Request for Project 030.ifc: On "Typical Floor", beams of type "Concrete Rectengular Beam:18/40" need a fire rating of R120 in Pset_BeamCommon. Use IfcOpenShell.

First a look at what the model holds.

```python
import ifcopenshell
import ifcopenshell.util.element

model = ifcopenshell.open("Project 030.ifc")
print(model.schema)
storey = next(s for s in model.by_type("IfcBuildingStorey") if s.Name == "Typical Floor")
beams = [e for e in ifcopenshell.util.element.get_decomposition(storey) if e.is_a("IfcBeam")]
seen = {}
for e in beams:
    element_type = ifcopenshell.util.element.get_type(e)
    key = (element_type.Name if element_type != e and element_type else None, ifcopenshell.util.element.get_pset(e, "Pset_BeamCommon", "FireRating"))
    seen[key] = seen.get(key, 0) + 1
for (name, value), count in sorted(seen.items(), key=str):
    print(count, "x", name, "|", value)
```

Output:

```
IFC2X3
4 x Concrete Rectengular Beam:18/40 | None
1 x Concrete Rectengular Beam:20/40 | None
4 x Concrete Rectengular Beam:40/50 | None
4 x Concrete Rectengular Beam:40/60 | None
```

```python
import ifcopenshell
import ifcopenshell.api.pset
import ifcopenshell.util.element

model = ifcopenshell.open("Project 030.ifc")

storey = next(s for s in model.by_type("IfcBuildingStorey") if s.Name == "Typical Floor")
beams = [e for e in ifcopenshell.util.element.get_decomposition(storey) if e.is_a("IfcBeam")]

count = 0
for e in beams:
    element_type = ifcopenshell.util.element.get_type(e)
    if element_type in (None, e) or element_type.Name != "Concrete Rectengular Beam:18/40":
        continue
    # add_pset returns the element's existing set when there is one.
    pset = ifcopenshell.api.pset.add_pset(model, product=e, name="Pset_BeamCommon")
    ifcopenshell.api.pset.edit_pset(model, pset=pset, properties={"FireRating": "R120"})
    count += 1

print(count, "beams updated")

model.write("Project 030_v2.ifc")
```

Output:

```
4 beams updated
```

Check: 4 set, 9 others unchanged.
